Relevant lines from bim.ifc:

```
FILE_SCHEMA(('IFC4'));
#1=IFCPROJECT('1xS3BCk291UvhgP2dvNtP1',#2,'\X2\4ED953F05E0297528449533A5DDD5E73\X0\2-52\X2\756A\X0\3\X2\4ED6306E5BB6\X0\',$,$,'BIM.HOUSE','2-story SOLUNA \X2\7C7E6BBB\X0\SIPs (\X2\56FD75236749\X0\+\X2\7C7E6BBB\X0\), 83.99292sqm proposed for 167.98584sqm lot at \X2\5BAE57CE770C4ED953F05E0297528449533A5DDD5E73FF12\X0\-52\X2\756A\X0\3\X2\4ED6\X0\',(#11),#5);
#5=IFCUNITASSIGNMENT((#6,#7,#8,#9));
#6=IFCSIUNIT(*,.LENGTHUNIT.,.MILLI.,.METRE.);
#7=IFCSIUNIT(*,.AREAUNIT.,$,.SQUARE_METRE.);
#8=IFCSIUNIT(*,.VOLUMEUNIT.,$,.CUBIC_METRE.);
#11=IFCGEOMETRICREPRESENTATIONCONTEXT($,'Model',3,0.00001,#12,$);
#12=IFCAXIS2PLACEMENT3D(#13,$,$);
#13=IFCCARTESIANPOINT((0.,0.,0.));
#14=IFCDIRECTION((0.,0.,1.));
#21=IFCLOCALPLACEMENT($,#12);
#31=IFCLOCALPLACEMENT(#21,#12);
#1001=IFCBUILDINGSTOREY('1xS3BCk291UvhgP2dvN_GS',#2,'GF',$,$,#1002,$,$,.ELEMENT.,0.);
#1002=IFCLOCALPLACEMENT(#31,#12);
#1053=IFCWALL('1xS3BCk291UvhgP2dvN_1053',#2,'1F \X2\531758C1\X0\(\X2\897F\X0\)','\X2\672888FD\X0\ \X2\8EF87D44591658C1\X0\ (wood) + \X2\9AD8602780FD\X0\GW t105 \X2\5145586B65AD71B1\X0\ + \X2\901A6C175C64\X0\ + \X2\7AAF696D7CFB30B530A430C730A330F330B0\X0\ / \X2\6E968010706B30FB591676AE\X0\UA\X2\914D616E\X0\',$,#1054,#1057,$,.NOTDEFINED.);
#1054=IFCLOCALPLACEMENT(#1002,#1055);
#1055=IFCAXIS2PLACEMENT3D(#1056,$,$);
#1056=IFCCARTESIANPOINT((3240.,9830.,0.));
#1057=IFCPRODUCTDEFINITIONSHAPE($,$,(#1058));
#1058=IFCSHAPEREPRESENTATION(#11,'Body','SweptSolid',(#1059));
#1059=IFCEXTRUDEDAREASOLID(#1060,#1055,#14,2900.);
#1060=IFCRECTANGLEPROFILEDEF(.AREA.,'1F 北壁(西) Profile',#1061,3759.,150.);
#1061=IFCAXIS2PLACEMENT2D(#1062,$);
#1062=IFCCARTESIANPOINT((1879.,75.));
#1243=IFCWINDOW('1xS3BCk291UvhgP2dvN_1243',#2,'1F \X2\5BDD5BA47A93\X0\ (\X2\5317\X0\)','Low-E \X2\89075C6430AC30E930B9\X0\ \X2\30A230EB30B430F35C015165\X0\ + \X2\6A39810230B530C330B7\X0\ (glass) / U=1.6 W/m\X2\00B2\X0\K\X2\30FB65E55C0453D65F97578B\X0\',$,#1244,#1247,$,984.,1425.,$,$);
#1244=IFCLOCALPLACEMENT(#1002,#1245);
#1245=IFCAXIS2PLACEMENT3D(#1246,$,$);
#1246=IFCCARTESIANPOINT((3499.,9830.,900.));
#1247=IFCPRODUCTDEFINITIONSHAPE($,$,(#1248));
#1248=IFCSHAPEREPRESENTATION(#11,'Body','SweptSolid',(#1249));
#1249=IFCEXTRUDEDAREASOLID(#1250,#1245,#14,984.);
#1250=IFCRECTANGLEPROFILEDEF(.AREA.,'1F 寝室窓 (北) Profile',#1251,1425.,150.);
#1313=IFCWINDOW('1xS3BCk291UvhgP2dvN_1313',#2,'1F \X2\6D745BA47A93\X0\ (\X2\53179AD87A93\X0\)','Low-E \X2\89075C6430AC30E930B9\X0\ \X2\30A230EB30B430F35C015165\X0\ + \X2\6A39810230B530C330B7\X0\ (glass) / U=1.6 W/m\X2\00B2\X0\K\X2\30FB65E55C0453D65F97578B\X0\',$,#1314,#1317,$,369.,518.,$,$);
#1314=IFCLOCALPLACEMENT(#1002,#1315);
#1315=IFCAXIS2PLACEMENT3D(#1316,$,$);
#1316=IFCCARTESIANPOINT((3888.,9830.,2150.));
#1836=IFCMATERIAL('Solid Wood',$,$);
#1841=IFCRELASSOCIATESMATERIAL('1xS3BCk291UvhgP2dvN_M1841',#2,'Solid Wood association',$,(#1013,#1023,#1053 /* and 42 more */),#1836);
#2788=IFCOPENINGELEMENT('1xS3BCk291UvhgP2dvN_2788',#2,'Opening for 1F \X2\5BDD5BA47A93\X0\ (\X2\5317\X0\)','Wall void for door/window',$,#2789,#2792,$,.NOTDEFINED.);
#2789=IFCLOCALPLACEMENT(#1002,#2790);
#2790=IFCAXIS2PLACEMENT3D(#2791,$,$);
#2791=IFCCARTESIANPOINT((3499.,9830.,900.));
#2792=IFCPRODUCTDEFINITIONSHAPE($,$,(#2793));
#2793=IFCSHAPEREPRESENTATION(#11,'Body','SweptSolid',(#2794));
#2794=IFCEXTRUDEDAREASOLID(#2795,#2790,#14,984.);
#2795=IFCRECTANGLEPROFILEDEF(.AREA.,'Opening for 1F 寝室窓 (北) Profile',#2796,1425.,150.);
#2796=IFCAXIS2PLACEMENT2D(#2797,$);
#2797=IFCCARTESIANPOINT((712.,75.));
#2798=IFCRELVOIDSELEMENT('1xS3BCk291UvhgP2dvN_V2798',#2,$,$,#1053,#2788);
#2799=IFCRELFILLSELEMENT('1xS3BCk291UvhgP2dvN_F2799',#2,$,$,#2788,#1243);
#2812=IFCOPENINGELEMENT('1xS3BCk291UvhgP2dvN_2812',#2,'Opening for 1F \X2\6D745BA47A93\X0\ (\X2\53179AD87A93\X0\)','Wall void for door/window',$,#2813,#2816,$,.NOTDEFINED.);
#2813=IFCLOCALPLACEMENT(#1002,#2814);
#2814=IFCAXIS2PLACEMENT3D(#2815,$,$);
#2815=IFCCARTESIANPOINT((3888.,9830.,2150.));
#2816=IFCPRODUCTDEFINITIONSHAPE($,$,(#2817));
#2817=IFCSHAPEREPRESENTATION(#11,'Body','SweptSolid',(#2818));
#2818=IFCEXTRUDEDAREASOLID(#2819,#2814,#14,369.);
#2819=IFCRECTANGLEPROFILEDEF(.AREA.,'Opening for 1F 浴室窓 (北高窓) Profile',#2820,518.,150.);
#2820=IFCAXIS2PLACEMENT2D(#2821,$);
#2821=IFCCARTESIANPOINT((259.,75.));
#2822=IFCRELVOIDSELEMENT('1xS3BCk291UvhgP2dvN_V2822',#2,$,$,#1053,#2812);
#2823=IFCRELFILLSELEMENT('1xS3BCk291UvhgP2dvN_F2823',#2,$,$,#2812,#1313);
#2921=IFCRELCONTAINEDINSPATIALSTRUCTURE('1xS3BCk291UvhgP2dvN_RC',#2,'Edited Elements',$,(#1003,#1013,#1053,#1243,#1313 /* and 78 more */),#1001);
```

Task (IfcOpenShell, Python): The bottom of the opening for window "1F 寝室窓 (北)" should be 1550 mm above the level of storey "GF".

```python
import numpy as np
import ifcopenshell
import ifcopenshell.api.geometry
import ifcopenshell.geom
import ifcopenshell.util.element
import ifcopenshell.util.placement
import ifcopenshell.util.shape
import ifcopenshell.util.unit

model = ifcopenshell.open("bim.ifc")
unit_scale = ifcopenshell.util.unit.calculate_unit_scale(model)

window = model.by_guid("1xS3BCk291UvhgP2dvN_1243")
opening = window.FillsVoids[0].RelatingOpeningElement
storey = ifcopenshell.util.element.get_container(window, ifc_class="IfcBuildingStorey")
level = ifcopenshell.util.placement.get_local_placement(storey.ObjectPlacement)[2, 3]

# The opening's origin need not be at the sill, so measure its lowest point.
shape = ifcopenshell.geom.create_shape(ifcopenshell.geom.settings(), opening)
bottom = ifcopenshell.util.shape.get_shape_bottom_elevation(shape, shape.geometry) / unit_scale
dz = level + 1.55 / unit_scale - bottom

shift = np.array([0.0, 0.0, dz])
# The window is not placed relative to its opening, so move both.
for product in (opening, window):
    matrix = ifcopenshell.util.placement.get_local_placement(product.ObjectPlacement)
    matrix[:3, 3] += shift
    ifcopenshell.api.geometry.edit_object_placement(model, product=product, matrix=matrix, is_si=False)

print(f"moved by {dz * unit_scale:+.3f} m")

model.write("bim_updated.ifc")
```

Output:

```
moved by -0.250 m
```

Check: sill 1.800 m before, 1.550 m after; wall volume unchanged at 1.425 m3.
